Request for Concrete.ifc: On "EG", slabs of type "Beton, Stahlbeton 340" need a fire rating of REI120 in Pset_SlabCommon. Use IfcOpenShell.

First a look at what the model holds.

```python
import ifcopenshell
import ifcopenshell.util.element

model = ifcopenshell.open("Concrete.ifc")
print(model.schema)
storey = next(s for s in model.by_type("IfcBuildingStorey") if s.Name == "EG")
slabs = [e for e in ifcopenshell.util.element.get_decomposition(storey) if e.is_a("IfcSlab")]
seen = {}
for e in slabs:
    element_type = ifcopenshell.util.element.get_type(e)
    key = (element_type.Name if element_type != e and element_type else None, ifcopenshell.util.element.get_pset(e, "Pset_SlabCommon", "FireRating"))
    seen[key] = seen.get(key, 0) + 1
for (name, value), count in sorted(seen.items(), key=str):
    print(count, "x", name, "|", value)
```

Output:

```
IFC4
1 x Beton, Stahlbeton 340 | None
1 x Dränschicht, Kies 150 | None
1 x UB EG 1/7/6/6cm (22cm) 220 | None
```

```python
import ifcopenshell
import ifcopenshell.api.pset
import ifcopenshell.util.element

model = ifcopenshell.open("Concrete.ifc")

storey = next(s for s in model.by_type("IfcBuildingStorey") if s.Name == "EG")
slabs = [e for e in ifcopenshell.util.element.get_decomposition(storey) if e.is_a("IfcSlab")]

count = 0
for e in slabs:
    element_type = ifcopenshell.util.element.get_type(e)
    if element_type in (None, e) or element_type.Name != "Beton, Stahlbeton 340":
        continue
    # add_pset returns the element's existing set when there is one.
    pset = ifcopenshell.api.pset.add_pset(model, product=e, name="Pset_SlabCommon")
    ifcopenshell.api.pset.edit_pset(model, pset=pset, properties={"FireRating": "REI120"})
    count += 1

print(count, "slabs updated")

model.write("Concrete_updated.ifc")
```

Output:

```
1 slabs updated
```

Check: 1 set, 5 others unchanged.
